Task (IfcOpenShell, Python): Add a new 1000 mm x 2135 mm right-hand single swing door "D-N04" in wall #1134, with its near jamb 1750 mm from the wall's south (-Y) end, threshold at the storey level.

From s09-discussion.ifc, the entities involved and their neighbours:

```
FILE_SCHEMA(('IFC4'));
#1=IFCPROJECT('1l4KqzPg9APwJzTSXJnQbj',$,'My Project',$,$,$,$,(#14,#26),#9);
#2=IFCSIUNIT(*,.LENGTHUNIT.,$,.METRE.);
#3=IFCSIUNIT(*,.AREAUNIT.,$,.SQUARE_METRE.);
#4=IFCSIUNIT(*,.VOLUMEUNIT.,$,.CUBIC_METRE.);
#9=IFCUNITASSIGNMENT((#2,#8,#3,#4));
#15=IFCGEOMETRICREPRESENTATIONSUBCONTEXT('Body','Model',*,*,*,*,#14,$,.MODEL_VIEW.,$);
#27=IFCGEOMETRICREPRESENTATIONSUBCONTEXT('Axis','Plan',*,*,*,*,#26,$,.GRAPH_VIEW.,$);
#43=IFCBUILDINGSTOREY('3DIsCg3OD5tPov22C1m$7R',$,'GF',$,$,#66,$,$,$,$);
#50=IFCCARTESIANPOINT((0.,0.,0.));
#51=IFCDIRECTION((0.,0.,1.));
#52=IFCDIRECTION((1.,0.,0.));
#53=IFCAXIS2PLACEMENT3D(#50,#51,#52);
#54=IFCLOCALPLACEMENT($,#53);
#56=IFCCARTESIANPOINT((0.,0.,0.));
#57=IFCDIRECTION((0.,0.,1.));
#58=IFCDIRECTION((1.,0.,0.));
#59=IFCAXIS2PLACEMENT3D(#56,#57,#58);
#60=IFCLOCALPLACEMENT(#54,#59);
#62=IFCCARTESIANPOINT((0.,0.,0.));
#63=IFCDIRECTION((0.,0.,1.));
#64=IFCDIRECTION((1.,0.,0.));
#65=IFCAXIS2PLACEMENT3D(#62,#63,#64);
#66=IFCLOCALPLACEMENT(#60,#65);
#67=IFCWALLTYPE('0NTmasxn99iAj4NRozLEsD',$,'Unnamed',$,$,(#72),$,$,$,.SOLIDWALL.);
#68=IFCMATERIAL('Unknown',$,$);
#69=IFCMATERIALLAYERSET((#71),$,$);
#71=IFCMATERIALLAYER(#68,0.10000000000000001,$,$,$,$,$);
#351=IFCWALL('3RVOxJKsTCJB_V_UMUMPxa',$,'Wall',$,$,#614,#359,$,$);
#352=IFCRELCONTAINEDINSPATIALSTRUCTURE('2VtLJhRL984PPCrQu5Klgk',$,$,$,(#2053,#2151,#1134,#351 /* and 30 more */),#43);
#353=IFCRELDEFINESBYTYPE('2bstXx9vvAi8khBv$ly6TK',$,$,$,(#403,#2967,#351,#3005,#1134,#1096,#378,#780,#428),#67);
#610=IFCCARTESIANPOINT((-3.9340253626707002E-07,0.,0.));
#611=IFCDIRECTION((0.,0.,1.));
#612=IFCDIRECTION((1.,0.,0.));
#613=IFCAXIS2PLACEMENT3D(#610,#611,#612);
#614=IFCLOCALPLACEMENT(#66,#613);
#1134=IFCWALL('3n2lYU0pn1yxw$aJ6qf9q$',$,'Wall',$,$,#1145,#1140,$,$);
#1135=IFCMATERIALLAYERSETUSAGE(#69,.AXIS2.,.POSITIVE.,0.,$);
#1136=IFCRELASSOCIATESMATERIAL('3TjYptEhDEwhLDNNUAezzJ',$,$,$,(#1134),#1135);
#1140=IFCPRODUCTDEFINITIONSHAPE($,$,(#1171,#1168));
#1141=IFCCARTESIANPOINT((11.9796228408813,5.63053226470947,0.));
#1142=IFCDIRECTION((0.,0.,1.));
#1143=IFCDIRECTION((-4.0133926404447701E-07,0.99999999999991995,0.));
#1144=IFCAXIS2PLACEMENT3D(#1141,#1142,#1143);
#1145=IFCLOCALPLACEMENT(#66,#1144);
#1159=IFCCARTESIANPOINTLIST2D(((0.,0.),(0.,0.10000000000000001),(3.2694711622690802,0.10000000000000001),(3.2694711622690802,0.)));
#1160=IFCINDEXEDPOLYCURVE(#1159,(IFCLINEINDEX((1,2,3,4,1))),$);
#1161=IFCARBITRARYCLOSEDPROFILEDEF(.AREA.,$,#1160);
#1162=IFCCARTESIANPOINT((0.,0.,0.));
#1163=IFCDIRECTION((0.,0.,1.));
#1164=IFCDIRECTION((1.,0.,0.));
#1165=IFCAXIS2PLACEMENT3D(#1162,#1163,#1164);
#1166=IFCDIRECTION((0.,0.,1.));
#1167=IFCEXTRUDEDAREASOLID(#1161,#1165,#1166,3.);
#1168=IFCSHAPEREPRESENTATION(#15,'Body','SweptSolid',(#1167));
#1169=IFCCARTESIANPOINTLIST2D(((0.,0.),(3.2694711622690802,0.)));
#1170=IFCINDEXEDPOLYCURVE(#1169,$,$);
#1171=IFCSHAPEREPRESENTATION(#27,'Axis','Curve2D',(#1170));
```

```python
import numpy as np
import ifcopenshell
import ifcopenshell.api.feature
import ifcopenshell.api.geometry
import ifcopenshell.api.root
import ifcopenshell.api.spatial
import ifcopenshell.geom
import ifcopenshell.util.element
import ifcopenshell.util.placement
import ifcopenshell.util.representation
import ifcopenshell.util.shape
import ifcopenshell.util.unit

model = ifcopenshell.open("s09-discussion.ifc")
unit_scale = ifcopenshell.util.unit.calculate_unit_scale(model)
settings = ifcopenshell.geom.settings()


def volume(element):
    """Net volume in cubic metres, openings subtracted."""
    shape = ifcopenshell.geom.create_shape(settings, element)
    return ifcopenshell.util.shape.get_volume(shape.geometry)


wall = model.by_guid("3n2lYU0pn1yxw$aJ6qf9q$")
storey = ifcopenshell.util.element.get_container(wall, ifc_class="IfcBuildingStorey")
context = ifcopenshell.util.representation.get_context(model, "Model", "Body", "MODEL_VIEW")
before = volume(wall)

width, height, from_end, sill = 1, 2.135, 1.75, 0.0  # metres

# The wall runs along its own X axis, and the end named is its -X end.
wall_shape = ifcopenshell.geom.create_shape(settings, wall)
x, y, z = ifcopenshell.util.shape.get_vertices(wall_shape.geometry).T
start = x.min() + from_end
face, thickness = float(y.min()), float(y.max() - y.min())
wall_matrix = ifcopenshell.util.placement.get_local_placement(wall.ObjectPlacement)
level = ifcopenshell.util.placement.get_local_placement(storey.ObjectPlacement)[2, 3]


def in_wall(x, y):
    """Placement at x, y metres in the wall's axes, at sill height."""
    matrix = wall_matrix.copy()
    matrix[:, 3] = wall_matrix @ np.array([x / unit_scale, y / unit_scale, 0.0, 1.0])
    matrix[2, 3] = level + sill / unit_scale
    return matrix


# Opening: a box that overshoots both wall faces by 50 mm.
opening = ifcopenshell.api.root.create_entity(model, ifc_class="IfcOpeningElement", predefined_type="OPENING")
box = ifcopenshell.api.geometry.add_wall_representation(
    model, context=context, length=width, height=height, thickness=thickness + 0.1
)
ifcopenshell.api.geometry.assign_representation(model, product=opening, representation=box)
ifcopenshell.api.geometry.edit_object_placement(model, product=opening, matrix=in_wall(start, face - 0.05), is_si=False)
ifcopenshell.api.feature.add_feature(model, feature=opening, element=wall)

door = ifcopenshell.api.root.create_entity(model, ifc_class="IfcDoor", name="D-N04", predefined_type="DOOR")
door.OverallWidth, door.OverallHeight = width / unit_scale, height / unit_scale
door.OperationType = "SINGLE_SWING_RIGHT"
body = ifcopenshell.api.geometry.add_door_representation(
    model,
    context=context,
    overall_width=door.OverallWidth,
    overall_height=door.OverallHeight,
    operation_type="SINGLE_SWING_RIGHT",
    lining_properties={"LiningDepth": thickness / unit_scale, "ThresholdDepth": thickness / unit_scale},
)
ifcopenshell.api.geometry.assign_representation(model, product=door, representation=body)
ifcopenshell.api.spatial.assign_container(model, products=[door], relating_structure=storey)
ifcopenshell.api.feature.add_filling(model, opening=opening, element=door)

# The lining spans the wall, so the door starts at the wall face.
ifcopenshell.api.geometry.edit_object_placement(model, product=door, matrix=in_wall(start, face), is_si=False)

after = volume(wall)

print(f"wall volume {before:.3f} -> {after:.3f} m3")

model.write("s09-discussion_v2.ifc")
```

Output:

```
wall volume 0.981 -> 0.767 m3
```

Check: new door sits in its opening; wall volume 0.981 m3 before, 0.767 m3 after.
